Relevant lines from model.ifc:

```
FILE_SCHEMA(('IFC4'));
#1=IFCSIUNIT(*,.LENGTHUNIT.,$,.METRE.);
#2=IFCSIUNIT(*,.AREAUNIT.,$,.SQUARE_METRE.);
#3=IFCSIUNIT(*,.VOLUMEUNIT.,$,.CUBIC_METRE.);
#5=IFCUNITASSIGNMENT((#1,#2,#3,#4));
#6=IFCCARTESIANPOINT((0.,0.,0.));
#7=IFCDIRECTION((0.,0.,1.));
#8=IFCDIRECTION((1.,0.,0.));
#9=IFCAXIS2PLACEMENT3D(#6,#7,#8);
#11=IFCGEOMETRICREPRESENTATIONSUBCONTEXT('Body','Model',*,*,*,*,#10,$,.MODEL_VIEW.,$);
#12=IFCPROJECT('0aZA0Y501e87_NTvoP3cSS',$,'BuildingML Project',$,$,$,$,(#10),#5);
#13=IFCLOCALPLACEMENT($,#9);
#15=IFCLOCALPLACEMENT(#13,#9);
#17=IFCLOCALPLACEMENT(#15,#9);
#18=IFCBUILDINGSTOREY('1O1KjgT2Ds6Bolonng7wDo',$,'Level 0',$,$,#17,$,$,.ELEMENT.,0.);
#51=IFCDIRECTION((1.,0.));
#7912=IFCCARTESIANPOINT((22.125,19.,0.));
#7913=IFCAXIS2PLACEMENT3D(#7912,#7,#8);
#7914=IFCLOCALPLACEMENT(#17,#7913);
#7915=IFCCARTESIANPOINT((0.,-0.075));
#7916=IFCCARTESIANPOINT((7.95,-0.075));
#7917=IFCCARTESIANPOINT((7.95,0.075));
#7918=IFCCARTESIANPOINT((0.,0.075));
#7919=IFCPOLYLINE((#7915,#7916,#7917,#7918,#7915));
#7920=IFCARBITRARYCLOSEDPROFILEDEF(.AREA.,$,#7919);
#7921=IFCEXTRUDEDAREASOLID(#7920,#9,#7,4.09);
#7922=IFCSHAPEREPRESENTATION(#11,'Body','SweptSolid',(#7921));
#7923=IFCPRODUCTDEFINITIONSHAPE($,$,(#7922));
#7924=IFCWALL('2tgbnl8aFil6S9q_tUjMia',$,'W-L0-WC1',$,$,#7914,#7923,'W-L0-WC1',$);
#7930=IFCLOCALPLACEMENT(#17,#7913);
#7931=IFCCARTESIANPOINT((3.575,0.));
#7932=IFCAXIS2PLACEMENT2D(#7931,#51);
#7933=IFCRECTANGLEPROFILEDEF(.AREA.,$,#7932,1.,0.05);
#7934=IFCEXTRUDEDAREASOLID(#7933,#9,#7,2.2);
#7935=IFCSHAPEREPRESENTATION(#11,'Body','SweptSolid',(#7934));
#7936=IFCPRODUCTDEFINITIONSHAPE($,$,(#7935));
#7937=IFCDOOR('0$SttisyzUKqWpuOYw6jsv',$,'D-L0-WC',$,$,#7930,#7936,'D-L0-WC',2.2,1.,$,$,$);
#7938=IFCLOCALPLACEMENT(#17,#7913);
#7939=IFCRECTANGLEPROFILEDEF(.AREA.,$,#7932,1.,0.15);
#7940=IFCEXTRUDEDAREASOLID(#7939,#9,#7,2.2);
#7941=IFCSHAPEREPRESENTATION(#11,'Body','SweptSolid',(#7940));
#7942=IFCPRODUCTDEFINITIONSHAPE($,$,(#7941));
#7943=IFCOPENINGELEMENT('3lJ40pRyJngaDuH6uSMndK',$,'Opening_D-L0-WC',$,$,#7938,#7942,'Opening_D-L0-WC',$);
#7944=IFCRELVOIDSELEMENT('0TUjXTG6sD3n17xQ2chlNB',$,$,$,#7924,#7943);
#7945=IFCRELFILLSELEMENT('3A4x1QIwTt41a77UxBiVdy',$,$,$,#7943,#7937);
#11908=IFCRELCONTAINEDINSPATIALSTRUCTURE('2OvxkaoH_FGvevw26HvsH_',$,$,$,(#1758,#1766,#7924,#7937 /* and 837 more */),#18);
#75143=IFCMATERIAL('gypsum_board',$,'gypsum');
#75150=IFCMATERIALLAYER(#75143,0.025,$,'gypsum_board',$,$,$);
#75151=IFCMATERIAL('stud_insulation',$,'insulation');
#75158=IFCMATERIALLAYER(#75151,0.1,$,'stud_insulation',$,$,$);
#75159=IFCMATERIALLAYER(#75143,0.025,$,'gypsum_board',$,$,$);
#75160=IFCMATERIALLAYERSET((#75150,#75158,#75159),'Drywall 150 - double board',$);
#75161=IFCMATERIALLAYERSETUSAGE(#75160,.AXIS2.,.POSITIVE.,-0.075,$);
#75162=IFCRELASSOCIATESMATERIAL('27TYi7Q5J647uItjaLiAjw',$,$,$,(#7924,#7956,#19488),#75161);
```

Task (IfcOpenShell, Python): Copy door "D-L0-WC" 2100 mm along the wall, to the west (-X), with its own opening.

```python
import ifcopenshell
import ifcopenshell.api.feature
import ifcopenshell.api.geometry
import ifcopenshell.api.root
import ifcopenshell.geom
import ifcopenshell.util.element
import ifcopenshell.util.placement
import ifcopenshell.util.shape
import ifcopenshell.util.unit

model = ifcopenshell.open("model.ifc")
unit_scale = ifcopenshell.util.unit.calculate_unit_scale(model)
settings = ifcopenshell.geom.settings()


def volume(element):
    """Net volume in cubic metres, openings subtracted."""
    shape = ifcopenshell.geom.create_shape(settings, element)
    return ifcopenshell.util.shape.get_volume(shape.geometry)


door = model.by_id(7937)
opening = door.FillsVoids[0].RelatingOpeningElement
wall = opening.VoidsElements[0].RelatingBuildingElement
before = volume(wall)
shift = ifcopenshell.util.placement.get_local_placement(wall.ObjectPlacement)[:3, 0] * -2.1 / unit_scale

# copy_class copies the void relationship, type, container and properties, but no geometry.
new_opening = ifcopenshell.api.root.copy_class(model, product=opening)
new_opening.Representation = ifcopenshell.util.element.copy_deep(
    model, opening.Representation, exclude=["IfcGeometricRepresentationContext", "IfcRepresentationMap"]
)
new_opening.Tag = None
new_door = ifcopenshell.api.root.copy_class(model, product=door)
new_door.Representation = ifcopenshell.util.element.copy_deep(
    model, door.Representation, exclude=["IfcGeometricRepresentationContext", "IfcRepresentationMap"]
)
new_door.Tag = None
ifcopenshell.api.feature.add_filling(model, opening=new_opening, element=new_door)

for old, new in ((opening, new_opening), (door, new_door)):
    matrix = ifcopenshell.util.placement.get_local_placement(old.ObjectPlacement)
    matrix[:3, 3] += shift
    ifcopenshell.api.geometry.edit_object_placement(model, product=new, matrix=matrix, is_si=False)

after = volume(wall)

print(f"wall volume {before:.3f} -> {after:.3f} m3")

model.write("model_v2.ifc")
```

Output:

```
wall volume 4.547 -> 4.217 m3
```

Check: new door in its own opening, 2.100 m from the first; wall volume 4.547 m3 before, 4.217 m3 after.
